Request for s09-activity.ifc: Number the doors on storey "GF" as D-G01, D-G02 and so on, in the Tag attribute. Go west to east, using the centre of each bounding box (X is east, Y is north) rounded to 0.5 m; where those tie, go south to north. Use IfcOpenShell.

First a look at what the model holds.

```python
import ifcopenshell
import ifcopenshell.util.element
import ifcopenshell.util.placement

model = ifcopenshell.open("s09-activity.ifc")
print(model.schema)
storey = next(s for s in model.by_type("IfcBuildingStorey") if s.Name == "GF")
doors = [e for e in ifcopenshell.util.element.get_decomposition(storey) if e.is_a("IfcDoor")]
for e in sorted(doors, key=lambda e: e.id()):
    origin = ifcopenshell.util.placement.get_local_placement(e.ObjectPlacement)[:3, 3]
    print(e.id(), e.Tag, e.Name, origin.round(2) + 0.0, sep=" | ")
```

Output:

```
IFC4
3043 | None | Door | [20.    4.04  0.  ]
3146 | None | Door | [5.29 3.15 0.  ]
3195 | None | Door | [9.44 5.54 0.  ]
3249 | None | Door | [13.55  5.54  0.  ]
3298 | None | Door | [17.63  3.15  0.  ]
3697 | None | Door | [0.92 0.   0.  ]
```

```python
import ifcopenshell
import ifcopenshell.geom
import ifcopenshell.util.element
import ifcopenshell.util.shape

model = ifcopenshell.open("s09-activity.ifc")
settings = ifcopenshell.geom.settings()
settings.set("use-world-coords", True)


def centre(element):
    shape = ifcopenshell.geom.create_shape(settings, element)
    return ifcopenshell.util.shape.get_bbox_centroid(shape.geometry)


storey = next(s for s in model.by_type("IfcBuildingStorey") if s.Name == "GF")
doors = [e for e in ifcopenshell.util.element.get_decomposition(storey) if e.is_a("IfcDoor")]

# Insertion points can sit at a corner or the storey origin, so sort by the geometry (in metres).
centres = {e: centre(e) for e in doors}
doors.sort(key=lambda e: (round(centres[e][0] / 0.5), centres[e][1]))

for i, e in enumerate(doors, start=1):
    number = f"D-G{i:02d}"
    e.Tag = number
    print(e.id(), number)

model.write("s09-activity_edited.ifc")
```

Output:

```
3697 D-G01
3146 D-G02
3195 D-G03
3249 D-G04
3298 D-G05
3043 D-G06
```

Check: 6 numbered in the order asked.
